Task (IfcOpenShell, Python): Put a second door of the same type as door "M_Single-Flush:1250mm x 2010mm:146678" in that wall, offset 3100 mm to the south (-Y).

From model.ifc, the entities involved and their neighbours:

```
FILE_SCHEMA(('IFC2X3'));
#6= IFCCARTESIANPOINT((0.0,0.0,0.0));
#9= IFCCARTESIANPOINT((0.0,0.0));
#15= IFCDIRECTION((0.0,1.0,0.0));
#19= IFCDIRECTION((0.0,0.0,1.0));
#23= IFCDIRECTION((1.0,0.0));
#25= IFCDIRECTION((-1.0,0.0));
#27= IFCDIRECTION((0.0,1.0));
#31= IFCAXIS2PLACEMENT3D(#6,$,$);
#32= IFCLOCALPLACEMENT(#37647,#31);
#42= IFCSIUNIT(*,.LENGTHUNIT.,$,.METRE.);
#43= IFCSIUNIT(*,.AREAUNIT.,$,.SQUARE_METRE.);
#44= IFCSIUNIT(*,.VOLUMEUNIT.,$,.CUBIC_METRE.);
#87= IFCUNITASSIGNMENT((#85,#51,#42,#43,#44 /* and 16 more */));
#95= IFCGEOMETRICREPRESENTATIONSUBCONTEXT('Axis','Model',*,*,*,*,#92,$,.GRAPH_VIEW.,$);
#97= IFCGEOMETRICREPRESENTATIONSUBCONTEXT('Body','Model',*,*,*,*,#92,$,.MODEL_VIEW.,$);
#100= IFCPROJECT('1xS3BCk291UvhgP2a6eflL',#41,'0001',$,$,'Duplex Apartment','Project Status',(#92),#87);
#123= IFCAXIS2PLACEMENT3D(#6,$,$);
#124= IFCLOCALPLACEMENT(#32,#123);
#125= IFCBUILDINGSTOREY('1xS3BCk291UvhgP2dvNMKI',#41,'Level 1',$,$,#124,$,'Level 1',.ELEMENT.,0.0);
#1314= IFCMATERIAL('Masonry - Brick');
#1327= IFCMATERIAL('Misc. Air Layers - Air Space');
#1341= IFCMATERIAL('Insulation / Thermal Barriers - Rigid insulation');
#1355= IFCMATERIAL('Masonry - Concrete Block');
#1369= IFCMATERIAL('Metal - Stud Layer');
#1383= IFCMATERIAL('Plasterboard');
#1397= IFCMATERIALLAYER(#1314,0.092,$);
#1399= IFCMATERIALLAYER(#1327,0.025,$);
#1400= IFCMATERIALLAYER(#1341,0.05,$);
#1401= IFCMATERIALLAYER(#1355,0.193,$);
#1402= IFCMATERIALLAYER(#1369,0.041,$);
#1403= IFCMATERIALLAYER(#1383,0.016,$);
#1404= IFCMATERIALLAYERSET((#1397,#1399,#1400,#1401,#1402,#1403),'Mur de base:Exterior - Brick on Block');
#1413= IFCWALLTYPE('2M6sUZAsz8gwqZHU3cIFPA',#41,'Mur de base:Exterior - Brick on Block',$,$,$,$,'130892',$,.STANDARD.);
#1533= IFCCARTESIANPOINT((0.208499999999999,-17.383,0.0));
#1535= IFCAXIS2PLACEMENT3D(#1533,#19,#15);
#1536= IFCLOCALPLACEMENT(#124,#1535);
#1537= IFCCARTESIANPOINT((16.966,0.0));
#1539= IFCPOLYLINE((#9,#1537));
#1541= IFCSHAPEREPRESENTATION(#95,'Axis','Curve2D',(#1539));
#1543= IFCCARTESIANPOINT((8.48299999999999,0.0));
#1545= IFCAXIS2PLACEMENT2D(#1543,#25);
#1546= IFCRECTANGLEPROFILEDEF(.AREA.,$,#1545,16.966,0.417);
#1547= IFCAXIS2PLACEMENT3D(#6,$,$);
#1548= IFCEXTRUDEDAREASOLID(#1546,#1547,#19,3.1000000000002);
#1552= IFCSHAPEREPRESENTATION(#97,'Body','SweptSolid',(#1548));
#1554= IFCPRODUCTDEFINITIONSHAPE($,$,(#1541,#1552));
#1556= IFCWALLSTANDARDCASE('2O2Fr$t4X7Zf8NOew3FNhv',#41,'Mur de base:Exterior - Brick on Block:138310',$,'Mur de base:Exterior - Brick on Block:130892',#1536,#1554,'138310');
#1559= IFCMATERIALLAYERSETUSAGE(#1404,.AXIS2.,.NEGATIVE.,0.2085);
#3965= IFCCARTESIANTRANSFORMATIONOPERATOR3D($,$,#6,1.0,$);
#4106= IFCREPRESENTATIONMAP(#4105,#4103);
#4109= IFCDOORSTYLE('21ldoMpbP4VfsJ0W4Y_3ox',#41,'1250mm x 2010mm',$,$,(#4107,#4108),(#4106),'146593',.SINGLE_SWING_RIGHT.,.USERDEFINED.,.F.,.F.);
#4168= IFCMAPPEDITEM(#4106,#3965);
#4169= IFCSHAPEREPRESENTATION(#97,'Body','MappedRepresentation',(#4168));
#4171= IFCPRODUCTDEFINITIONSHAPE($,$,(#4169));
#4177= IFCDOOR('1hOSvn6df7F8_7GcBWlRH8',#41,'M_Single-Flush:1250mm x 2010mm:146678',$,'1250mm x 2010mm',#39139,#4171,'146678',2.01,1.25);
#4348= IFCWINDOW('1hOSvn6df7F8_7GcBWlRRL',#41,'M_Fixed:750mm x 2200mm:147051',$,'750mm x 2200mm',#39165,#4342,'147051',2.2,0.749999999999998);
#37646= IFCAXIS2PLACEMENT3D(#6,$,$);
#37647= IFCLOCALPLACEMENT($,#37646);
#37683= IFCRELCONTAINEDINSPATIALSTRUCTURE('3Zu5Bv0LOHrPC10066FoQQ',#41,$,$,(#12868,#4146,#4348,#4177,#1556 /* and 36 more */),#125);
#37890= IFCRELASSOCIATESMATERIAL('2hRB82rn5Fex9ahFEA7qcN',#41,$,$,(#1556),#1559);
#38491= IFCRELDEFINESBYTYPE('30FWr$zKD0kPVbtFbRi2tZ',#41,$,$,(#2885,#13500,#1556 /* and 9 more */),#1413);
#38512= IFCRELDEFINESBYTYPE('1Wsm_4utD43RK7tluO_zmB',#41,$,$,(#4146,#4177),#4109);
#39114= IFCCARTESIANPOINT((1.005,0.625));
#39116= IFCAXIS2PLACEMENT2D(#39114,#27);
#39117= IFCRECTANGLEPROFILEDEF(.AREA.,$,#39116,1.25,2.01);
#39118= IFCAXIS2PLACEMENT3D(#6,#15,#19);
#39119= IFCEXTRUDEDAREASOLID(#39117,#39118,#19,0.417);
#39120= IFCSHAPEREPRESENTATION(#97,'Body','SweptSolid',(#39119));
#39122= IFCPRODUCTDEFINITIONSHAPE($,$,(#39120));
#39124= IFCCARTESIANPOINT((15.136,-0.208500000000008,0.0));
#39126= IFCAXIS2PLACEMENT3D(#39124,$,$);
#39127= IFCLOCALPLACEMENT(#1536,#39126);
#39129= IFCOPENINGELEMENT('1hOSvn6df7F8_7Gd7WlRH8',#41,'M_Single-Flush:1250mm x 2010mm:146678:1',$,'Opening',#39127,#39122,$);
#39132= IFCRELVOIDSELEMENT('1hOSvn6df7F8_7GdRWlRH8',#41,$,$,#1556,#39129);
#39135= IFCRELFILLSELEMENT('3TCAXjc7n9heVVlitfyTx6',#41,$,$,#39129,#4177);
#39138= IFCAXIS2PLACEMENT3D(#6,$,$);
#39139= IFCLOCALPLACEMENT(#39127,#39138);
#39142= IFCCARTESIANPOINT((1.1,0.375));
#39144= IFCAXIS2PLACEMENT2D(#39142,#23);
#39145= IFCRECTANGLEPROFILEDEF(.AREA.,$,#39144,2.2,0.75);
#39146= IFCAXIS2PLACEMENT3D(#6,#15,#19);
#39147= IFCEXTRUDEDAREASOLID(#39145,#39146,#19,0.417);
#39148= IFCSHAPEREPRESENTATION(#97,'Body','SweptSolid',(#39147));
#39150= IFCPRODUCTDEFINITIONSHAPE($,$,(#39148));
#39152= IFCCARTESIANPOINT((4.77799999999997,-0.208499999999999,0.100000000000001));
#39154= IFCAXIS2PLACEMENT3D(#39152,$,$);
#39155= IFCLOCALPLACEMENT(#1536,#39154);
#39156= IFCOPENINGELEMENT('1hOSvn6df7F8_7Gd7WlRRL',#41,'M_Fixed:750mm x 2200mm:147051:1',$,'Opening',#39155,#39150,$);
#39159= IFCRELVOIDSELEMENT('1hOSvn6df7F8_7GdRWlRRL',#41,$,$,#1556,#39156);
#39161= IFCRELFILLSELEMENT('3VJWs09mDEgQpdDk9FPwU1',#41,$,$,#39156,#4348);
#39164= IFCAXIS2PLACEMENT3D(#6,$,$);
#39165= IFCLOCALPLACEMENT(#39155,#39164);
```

```python
import ifcopenshell
import ifcopenshell.api.feature
import ifcopenshell.api.geometry
import ifcopenshell.api.root
import ifcopenshell.geom
import ifcopenshell.util.element
import ifcopenshell.util.placement
import ifcopenshell.util.shape
import ifcopenshell.util.unit

model = ifcopenshell.open("model.ifc")
unit_scale = ifcopenshell.util.unit.calculate_unit_scale(model)
settings = ifcopenshell.geom.settings()


def volume(element):
    """Net volume in cubic metres, openings subtracted."""
    shape = ifcopenshell.geom.create_shape(settings, element)
    return ifcopenshell.util.shape.get_volume(shape.geometry)


def reuse_history(source, copy):
    """copy_class also copies each property set's owner history, people and application; keep the originals."""
    for rel in copy.IsDefinedBy:
        if rel.is_a("IfcRelDefinesByProperties") and (history := rel.RelatingPropertyDefinition.OwnerHistory):
            rel.RelatingPropertyDefinition.OwnerHistory = source.OwnerHistory
            ifcopenshell.util.element.remove_deep2(model, history)


door = model.by_guid("1hOSvn6df7F8_7GcBWlRH8")
opening = door.FillsVoids[0].RelatingOpeningElement
wall = opening.VoidsElements[0].RelatingBuildingElement
before = volume(wall)
shift = ifcopenshell.util.placement.get_local_placement(wall.ObjectPlacement)[:3, 0] * -3.1 / unit_scale

# copy_class copies the void relationship, type, container and properties, but no geometry.
new_opening = ifcopenshell.api.root.copy_class(model, product=opening)
new_opening.Representation = ifcopenshell.util.element.copy_deep(
    model, opening.Representation, exclude=["IfcGeometricRepresentationContext", "IfcRepresentationMap"]
)
new_opening.Name = "M_Single-Flush:1250mm x 2010mm"
new_door = ifcopenshell.api.root.copy_class(model, product=door)
new_door.Representation = ifcopenshell.util.element.copy_deep(
    model, door.Representation, exclude=["IfcGeometricRepresentationContext", "IfcRepresentationMap"]
)
new_door.Name = "M_Single-Flush:1250mm x 2010mm"
new_door.Tag = None
reuse_history(door, new_door)
fills = ifcopenshell.api.feature.add_filling(model, opening=new_opening, element=new_door)
fills.OwnerHistory = new_door.OwnerHistory  # required in IFC2X3

for old, new in ((opening, new_opening), (door, new_door)):
    matrix = ifcopenshell.util.placement.get_local_placement(old.ObjectPlacement)
    matrix[:3, 3] += shift
    ifcopenshell.api.geometry.edit_object_placement(model, product=new, matrix=matrix, is_si=False)

after = volume(wall)

print(f"wall volume {before:.3f} -> {after:.3f} m3")

model.write("model_v2.ifc")
```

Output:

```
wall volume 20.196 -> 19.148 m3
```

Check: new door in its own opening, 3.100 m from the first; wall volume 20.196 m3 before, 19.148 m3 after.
